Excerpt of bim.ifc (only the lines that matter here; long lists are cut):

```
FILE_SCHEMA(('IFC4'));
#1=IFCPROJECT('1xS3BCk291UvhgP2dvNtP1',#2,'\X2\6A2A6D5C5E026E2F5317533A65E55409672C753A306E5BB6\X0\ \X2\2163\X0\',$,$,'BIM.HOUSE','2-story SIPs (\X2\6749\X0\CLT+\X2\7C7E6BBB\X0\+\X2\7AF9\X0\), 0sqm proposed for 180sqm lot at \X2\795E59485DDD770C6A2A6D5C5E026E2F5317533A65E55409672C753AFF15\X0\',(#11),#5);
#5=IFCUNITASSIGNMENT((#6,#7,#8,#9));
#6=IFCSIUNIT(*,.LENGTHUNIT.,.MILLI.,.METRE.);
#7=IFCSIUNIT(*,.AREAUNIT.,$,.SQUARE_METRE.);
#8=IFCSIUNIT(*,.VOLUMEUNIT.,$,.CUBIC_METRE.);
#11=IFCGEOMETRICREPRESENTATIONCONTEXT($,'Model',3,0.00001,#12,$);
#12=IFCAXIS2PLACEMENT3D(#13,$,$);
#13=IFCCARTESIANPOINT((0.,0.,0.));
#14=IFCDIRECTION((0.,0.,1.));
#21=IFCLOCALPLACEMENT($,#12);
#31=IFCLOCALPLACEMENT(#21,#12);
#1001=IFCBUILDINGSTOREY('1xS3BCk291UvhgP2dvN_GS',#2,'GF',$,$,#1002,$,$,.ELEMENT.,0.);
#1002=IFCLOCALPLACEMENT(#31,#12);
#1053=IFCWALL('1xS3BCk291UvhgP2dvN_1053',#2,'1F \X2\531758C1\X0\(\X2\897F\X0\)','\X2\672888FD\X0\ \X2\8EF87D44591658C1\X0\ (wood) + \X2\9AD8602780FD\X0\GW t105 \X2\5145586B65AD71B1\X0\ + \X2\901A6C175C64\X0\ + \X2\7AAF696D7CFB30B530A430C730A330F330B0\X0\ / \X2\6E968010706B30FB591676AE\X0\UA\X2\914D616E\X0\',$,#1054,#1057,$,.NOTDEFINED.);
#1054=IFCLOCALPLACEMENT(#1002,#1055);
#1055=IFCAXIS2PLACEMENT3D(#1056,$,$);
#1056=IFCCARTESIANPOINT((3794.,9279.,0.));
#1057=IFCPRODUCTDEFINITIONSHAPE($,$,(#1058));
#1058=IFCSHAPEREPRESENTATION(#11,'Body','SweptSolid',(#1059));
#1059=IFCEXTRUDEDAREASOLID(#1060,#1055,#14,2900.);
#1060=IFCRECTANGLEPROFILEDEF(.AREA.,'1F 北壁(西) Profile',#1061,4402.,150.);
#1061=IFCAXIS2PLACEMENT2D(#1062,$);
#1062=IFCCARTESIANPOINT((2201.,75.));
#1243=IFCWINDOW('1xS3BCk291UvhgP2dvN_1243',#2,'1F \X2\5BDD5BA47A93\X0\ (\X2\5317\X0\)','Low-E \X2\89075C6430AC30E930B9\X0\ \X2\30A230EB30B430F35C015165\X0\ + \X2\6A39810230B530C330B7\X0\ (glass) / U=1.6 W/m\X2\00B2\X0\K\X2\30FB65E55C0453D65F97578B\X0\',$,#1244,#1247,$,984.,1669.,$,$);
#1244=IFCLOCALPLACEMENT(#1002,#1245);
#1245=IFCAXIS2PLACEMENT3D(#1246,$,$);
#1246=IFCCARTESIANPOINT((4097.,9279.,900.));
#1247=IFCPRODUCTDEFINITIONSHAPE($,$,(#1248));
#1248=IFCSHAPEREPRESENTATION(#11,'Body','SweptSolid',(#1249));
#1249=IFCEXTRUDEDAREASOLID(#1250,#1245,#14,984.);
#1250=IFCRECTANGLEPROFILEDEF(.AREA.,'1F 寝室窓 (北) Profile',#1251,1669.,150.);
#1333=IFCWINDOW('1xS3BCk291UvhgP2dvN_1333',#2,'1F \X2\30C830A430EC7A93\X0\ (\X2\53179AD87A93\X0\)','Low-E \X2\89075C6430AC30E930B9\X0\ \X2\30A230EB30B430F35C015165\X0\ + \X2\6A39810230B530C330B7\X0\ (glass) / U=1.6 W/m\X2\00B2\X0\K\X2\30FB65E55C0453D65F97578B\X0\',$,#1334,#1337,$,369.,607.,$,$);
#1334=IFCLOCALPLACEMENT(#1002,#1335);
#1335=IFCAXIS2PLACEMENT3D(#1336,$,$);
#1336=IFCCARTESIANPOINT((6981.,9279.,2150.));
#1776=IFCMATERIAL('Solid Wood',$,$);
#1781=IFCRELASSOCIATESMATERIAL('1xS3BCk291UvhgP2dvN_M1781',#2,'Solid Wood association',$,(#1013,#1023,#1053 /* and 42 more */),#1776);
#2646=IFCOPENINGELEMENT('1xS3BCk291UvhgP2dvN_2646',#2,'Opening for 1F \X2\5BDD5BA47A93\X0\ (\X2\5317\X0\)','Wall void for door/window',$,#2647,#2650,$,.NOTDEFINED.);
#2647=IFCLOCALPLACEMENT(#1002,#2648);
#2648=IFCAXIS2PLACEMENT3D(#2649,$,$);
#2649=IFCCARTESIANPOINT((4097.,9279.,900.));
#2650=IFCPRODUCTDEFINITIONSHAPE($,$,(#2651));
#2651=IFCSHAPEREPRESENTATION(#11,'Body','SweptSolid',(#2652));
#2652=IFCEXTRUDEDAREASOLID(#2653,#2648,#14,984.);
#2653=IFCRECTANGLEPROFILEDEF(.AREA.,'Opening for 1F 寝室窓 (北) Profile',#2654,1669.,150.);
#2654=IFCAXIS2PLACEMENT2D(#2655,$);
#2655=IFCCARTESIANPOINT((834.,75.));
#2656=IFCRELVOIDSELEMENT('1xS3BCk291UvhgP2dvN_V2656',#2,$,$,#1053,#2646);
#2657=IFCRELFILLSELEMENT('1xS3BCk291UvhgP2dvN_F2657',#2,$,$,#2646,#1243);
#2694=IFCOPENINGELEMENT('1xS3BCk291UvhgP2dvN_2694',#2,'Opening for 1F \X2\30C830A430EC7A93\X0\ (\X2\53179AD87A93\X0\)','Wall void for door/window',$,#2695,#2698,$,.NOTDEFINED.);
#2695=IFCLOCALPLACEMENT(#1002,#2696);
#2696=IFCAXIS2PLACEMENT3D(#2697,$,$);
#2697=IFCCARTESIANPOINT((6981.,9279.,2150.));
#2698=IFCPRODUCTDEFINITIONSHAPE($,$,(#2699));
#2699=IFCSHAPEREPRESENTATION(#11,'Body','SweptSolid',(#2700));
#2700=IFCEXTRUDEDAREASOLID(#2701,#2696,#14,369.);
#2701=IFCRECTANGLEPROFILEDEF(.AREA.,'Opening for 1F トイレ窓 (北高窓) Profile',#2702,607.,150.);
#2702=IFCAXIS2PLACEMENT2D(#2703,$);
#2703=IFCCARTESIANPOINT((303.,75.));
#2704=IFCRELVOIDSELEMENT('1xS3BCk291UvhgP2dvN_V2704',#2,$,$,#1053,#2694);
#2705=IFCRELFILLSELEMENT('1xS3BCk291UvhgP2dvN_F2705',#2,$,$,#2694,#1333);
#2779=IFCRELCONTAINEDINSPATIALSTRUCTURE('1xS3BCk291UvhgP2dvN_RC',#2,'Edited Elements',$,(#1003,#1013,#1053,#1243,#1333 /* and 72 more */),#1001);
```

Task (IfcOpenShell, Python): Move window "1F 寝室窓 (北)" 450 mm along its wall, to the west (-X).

```python
import ifcopenshell
import ifcopenshell.api.geometry
import ifcopenshell.util.placement
import ifcopenshell.util.unit

model = ifcopenshell.open("bim.ifc")
unit_scale = ifcopenshell.util.unit.calculate_unit_scale(model)

window = model.by_guid("1xS3BCk291UvhgP2dvN_1243")
opening = window.FillsVoids[0].RelatingOpeningElement
wall = opening.VoidsElements[0].RelatingBuildingElement

wall_matrix = ifcopenshell.util.placement.get_local_placement(wall.ObjectPlacement)
shift = wall_matrix[:3, 0] * -0.45 / unit_scale
before = ifcopenshell.util.placement.get_local_placement(window.ObjectPlacement)[:3, 3].copy()

# The window is not placed relative to its opening, so move both.
for product in (opening, window):
    matrix = ifcopenshell.util.placement.get_local_placement(product.ObjectPlacement)
    matrix[:3, 3] += shift
    ifcopenshell.api.geometry.edit_object_placement(model, product=product, matrix=matrix, is_si=False)

after = ifcopenshell.util.placement.get_local_placement(window.ObjectPlacement)[:3, 3]
print("window moved by", (after - before).round(3) + 0.0)

model.write("bim_v2.ifc")
```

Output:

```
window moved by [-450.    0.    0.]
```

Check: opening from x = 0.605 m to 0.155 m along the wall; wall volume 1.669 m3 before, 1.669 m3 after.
